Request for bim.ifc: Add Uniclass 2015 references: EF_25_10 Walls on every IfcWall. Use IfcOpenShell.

First a look at what the model holds.

```python
import ifcopenshell

model = ifcopenshell.open("bim.ifc")
print(model.schema)
print("classifications:", [c.Name for c in model.by_type("IfcClassification")])
for ifc_class in ("IfcDoor", "IfcRoof", "IfcStair", "IfcWall", "IfcWindow"):
    print(ifc_class, len(model.by_type(ifc_class)))
```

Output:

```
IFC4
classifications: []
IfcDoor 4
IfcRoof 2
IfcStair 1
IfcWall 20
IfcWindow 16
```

```python
import ifcopenshell
import ifcopenshell.api.classification

model = ifcopenshell.open("bim.ifc")

system = ifcopenshell.api.classification.add_classification(model, classification="Uniclass 2015")

codes = {
    "IfcWall": ("EF_25_10", "Walls"),
}
for ifc_class, (code, name) in codes.items():
    products = model.by_type(ifc_class)
    ifcopenshell.api.classification.add_reference(
        model, products=products, classification=system, identification=code, name=name
    )
    print(code, len(products))

model.write("bim_rev.ifc")
```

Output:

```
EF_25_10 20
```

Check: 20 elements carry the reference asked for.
